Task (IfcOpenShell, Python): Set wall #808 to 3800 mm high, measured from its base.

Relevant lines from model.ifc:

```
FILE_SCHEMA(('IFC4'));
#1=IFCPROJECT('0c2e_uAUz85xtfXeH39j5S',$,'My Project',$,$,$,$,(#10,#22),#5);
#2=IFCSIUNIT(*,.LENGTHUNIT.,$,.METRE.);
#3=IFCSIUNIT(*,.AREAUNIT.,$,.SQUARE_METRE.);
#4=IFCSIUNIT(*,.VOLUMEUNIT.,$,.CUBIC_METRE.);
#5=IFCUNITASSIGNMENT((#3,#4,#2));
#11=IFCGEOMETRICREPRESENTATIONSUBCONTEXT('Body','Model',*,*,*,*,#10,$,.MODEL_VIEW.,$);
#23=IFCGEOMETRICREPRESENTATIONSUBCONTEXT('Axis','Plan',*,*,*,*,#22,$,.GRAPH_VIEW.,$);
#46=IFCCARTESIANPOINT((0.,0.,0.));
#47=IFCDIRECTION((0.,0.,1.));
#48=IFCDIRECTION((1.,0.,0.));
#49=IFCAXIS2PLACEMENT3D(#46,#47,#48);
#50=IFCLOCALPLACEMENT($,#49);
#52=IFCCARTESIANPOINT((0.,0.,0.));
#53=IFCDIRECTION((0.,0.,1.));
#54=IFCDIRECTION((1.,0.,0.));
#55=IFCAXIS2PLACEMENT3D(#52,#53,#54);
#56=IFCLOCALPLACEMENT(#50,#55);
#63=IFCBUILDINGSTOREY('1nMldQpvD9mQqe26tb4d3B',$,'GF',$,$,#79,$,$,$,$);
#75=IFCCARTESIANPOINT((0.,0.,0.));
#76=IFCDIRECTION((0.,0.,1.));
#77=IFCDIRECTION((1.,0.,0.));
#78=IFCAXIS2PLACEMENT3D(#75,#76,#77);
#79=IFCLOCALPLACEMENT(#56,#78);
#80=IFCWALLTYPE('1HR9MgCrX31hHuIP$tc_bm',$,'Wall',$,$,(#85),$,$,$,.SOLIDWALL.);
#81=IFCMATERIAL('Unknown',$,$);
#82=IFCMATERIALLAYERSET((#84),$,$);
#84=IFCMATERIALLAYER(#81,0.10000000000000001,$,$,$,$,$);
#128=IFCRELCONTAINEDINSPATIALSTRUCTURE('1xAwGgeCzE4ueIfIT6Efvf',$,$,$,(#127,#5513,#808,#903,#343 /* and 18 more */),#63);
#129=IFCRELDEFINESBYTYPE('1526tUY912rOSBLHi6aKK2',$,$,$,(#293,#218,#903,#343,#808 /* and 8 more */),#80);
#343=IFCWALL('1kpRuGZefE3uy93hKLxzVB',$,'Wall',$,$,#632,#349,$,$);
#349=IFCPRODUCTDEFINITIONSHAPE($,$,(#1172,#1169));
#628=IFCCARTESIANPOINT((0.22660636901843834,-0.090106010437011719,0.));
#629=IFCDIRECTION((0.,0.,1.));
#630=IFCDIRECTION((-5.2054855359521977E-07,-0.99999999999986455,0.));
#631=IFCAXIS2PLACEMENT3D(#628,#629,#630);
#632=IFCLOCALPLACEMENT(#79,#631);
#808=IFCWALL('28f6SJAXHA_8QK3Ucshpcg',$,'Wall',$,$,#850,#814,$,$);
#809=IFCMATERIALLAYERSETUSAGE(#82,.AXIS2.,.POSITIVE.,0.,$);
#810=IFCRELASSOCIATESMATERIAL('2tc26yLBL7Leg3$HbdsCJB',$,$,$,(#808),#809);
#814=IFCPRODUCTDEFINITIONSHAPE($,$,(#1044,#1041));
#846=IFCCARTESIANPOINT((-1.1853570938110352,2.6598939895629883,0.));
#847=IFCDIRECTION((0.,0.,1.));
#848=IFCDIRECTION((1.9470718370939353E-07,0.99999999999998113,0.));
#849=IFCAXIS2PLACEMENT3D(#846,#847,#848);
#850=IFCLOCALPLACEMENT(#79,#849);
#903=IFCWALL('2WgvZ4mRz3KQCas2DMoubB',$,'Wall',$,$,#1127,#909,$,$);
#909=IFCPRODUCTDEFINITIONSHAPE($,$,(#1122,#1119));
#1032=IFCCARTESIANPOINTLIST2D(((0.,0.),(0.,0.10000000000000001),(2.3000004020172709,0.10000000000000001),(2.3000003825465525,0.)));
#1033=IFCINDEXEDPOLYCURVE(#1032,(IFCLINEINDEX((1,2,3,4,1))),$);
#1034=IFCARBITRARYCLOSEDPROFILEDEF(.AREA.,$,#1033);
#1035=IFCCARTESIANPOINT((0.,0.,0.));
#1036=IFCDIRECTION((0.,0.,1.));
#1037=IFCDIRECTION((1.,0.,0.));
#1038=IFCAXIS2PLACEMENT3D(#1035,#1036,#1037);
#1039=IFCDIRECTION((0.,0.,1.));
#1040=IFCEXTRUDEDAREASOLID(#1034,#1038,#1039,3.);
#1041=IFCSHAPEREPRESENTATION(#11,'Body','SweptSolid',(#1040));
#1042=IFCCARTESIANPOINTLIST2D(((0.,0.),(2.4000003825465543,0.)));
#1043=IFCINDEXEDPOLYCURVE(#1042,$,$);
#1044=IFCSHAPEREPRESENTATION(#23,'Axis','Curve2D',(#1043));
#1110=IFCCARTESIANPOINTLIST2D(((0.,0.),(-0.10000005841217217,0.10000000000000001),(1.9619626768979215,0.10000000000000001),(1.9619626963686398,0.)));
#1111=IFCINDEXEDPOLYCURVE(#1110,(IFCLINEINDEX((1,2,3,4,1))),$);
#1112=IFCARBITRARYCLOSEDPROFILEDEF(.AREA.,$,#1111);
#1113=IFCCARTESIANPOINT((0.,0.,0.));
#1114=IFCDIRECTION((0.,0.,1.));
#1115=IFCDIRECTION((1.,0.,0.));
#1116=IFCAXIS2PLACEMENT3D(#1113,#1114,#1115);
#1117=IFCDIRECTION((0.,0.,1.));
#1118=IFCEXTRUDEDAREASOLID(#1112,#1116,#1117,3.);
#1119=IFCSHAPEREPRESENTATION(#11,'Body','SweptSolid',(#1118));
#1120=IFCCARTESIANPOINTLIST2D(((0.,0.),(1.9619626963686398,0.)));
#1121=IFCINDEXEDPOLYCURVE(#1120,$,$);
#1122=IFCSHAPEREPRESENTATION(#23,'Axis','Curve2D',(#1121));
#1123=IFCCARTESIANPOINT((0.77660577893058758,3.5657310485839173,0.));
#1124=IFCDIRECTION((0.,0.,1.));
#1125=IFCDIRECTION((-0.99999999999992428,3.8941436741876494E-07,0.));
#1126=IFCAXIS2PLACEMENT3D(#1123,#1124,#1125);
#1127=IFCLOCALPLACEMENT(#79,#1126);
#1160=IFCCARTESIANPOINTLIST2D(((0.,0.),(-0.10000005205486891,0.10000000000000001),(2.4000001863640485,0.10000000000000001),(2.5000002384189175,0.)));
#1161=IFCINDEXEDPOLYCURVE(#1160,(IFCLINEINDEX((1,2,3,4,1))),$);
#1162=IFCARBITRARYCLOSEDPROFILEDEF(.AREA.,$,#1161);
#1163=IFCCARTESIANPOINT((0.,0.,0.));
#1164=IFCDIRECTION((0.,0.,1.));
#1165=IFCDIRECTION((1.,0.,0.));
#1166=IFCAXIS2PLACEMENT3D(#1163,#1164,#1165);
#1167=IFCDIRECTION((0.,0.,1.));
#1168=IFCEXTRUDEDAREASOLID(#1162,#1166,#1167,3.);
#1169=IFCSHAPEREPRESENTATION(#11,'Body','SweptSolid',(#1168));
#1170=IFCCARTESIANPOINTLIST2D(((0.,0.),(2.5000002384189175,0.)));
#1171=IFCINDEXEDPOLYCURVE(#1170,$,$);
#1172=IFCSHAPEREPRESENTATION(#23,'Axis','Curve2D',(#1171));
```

```python
import ifcopenshell
import ifcopenshell.geom
import ifcopenshell.util.representation
import ifcopenshell.util.shape

model = ifcopenshell.open("model.ifc")
settings = ifcopenshell.geom.settings()


def volume(element):
    """Net volume in cubic metres, openings subtracted."""
    shape = ifcopenshell.geom.create_shape(settings, element)
    return ifcopenshell.util.shape.get_volume(shape.geometry)


wall = model.by_id(808)
before = volume(wall)

body = ifcopenshell.util.representation.get_representation(wall, "Model", "Body")
solid = body.Items[0]
old_height = solid.Depth
solid.Depth = 3.8
after = volume(wall)

print(f"height {old_height:g} -> {solid.Depth:g}, volume {before:.3f} -> {after:.3f} m3")

model.write("model_edited.ifc")
```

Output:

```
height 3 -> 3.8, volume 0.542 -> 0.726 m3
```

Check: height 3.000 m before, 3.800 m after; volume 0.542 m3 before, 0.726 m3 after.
